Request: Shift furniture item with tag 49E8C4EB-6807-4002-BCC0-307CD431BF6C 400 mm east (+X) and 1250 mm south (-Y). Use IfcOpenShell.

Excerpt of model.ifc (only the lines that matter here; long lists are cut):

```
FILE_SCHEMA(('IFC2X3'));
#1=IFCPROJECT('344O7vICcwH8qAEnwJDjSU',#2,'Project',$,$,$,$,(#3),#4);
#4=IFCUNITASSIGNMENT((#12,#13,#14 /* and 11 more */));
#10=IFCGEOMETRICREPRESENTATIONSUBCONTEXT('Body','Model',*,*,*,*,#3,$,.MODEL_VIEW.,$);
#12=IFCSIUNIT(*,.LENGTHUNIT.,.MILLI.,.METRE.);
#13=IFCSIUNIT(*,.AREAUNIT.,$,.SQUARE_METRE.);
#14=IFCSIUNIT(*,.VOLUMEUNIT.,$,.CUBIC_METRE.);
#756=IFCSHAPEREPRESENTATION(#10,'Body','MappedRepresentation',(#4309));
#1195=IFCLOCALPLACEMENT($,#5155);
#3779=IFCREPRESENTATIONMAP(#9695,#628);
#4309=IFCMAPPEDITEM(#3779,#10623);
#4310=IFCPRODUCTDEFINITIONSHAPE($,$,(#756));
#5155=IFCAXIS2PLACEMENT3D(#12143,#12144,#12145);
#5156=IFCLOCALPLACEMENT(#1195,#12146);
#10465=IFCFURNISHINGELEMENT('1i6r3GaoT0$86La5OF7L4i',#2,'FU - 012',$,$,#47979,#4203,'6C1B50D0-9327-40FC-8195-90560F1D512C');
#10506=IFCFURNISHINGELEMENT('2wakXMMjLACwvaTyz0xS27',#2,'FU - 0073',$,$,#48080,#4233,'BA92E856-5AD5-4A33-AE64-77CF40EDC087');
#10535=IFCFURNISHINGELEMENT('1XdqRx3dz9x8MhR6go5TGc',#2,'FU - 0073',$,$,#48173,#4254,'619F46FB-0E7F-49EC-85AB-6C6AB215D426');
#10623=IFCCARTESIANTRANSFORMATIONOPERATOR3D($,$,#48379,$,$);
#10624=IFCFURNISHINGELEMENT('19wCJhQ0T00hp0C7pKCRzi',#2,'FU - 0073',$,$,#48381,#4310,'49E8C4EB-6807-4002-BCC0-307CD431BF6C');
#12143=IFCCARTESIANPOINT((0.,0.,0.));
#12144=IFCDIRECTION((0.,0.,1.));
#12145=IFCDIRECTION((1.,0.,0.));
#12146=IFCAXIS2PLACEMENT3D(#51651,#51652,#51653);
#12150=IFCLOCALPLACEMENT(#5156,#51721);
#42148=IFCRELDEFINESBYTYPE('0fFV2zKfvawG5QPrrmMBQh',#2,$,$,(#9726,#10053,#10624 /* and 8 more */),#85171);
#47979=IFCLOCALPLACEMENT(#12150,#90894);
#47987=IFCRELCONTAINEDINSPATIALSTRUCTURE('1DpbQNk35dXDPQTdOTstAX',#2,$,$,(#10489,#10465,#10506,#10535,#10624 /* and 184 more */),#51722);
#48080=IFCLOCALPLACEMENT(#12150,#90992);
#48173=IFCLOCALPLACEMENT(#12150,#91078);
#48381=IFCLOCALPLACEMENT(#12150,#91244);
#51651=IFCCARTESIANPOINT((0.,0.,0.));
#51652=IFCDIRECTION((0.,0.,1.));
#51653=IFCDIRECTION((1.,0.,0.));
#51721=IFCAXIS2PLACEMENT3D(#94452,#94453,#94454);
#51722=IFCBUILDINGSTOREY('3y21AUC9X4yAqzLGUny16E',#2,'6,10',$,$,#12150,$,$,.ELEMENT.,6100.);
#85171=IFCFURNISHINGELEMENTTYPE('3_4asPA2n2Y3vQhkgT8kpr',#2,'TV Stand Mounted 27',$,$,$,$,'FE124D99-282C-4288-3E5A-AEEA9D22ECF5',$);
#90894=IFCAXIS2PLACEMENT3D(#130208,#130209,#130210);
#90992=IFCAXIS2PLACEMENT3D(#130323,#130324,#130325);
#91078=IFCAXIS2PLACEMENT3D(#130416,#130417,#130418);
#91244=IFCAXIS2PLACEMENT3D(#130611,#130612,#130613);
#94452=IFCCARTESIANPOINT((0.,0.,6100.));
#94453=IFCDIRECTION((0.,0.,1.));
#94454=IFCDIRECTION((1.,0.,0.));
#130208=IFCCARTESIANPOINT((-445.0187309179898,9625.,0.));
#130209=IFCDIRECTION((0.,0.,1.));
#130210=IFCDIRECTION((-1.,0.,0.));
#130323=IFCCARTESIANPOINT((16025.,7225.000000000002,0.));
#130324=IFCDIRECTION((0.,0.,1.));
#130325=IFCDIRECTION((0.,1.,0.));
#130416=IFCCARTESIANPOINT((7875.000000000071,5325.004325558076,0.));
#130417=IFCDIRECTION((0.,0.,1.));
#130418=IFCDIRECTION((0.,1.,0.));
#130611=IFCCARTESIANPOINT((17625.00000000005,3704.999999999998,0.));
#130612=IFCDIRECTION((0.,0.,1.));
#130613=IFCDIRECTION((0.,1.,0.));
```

```python
import ifcopenshell
import ifcopenshell.api.geometry
import ifcopenshell.util.placement
import ifcopenshell.util.unit

model = ifcopenshell.open("model.ifc")
unit_scale = ifcopenshell.util.unit.calculate_unit_scale(model)

item = model.by_guid("19wCJhQ0T00hp0C7pKCRzi")
matrix = ifcopenshell.util.placement.get_local_placement(item.ObjectPlacement)
matrix[0, 3] += 0.4 / unit_scale
matrix[1, 3] -= 1.25 / unit_scale
ifcopenshell.api.geometry.edit_object_placement(model, product=item, matrix=matrix, is_si=False)

print(ifcopenshell.util.placement.get_local_placement(item.ObjectPlacement).round(3) + 0.0)

model.write("model-out.ifc")
```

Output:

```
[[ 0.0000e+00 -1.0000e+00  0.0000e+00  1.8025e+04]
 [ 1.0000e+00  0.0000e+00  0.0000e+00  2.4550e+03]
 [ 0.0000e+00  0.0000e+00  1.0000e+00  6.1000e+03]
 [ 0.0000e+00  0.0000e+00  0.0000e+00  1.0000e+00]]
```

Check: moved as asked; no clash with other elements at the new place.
